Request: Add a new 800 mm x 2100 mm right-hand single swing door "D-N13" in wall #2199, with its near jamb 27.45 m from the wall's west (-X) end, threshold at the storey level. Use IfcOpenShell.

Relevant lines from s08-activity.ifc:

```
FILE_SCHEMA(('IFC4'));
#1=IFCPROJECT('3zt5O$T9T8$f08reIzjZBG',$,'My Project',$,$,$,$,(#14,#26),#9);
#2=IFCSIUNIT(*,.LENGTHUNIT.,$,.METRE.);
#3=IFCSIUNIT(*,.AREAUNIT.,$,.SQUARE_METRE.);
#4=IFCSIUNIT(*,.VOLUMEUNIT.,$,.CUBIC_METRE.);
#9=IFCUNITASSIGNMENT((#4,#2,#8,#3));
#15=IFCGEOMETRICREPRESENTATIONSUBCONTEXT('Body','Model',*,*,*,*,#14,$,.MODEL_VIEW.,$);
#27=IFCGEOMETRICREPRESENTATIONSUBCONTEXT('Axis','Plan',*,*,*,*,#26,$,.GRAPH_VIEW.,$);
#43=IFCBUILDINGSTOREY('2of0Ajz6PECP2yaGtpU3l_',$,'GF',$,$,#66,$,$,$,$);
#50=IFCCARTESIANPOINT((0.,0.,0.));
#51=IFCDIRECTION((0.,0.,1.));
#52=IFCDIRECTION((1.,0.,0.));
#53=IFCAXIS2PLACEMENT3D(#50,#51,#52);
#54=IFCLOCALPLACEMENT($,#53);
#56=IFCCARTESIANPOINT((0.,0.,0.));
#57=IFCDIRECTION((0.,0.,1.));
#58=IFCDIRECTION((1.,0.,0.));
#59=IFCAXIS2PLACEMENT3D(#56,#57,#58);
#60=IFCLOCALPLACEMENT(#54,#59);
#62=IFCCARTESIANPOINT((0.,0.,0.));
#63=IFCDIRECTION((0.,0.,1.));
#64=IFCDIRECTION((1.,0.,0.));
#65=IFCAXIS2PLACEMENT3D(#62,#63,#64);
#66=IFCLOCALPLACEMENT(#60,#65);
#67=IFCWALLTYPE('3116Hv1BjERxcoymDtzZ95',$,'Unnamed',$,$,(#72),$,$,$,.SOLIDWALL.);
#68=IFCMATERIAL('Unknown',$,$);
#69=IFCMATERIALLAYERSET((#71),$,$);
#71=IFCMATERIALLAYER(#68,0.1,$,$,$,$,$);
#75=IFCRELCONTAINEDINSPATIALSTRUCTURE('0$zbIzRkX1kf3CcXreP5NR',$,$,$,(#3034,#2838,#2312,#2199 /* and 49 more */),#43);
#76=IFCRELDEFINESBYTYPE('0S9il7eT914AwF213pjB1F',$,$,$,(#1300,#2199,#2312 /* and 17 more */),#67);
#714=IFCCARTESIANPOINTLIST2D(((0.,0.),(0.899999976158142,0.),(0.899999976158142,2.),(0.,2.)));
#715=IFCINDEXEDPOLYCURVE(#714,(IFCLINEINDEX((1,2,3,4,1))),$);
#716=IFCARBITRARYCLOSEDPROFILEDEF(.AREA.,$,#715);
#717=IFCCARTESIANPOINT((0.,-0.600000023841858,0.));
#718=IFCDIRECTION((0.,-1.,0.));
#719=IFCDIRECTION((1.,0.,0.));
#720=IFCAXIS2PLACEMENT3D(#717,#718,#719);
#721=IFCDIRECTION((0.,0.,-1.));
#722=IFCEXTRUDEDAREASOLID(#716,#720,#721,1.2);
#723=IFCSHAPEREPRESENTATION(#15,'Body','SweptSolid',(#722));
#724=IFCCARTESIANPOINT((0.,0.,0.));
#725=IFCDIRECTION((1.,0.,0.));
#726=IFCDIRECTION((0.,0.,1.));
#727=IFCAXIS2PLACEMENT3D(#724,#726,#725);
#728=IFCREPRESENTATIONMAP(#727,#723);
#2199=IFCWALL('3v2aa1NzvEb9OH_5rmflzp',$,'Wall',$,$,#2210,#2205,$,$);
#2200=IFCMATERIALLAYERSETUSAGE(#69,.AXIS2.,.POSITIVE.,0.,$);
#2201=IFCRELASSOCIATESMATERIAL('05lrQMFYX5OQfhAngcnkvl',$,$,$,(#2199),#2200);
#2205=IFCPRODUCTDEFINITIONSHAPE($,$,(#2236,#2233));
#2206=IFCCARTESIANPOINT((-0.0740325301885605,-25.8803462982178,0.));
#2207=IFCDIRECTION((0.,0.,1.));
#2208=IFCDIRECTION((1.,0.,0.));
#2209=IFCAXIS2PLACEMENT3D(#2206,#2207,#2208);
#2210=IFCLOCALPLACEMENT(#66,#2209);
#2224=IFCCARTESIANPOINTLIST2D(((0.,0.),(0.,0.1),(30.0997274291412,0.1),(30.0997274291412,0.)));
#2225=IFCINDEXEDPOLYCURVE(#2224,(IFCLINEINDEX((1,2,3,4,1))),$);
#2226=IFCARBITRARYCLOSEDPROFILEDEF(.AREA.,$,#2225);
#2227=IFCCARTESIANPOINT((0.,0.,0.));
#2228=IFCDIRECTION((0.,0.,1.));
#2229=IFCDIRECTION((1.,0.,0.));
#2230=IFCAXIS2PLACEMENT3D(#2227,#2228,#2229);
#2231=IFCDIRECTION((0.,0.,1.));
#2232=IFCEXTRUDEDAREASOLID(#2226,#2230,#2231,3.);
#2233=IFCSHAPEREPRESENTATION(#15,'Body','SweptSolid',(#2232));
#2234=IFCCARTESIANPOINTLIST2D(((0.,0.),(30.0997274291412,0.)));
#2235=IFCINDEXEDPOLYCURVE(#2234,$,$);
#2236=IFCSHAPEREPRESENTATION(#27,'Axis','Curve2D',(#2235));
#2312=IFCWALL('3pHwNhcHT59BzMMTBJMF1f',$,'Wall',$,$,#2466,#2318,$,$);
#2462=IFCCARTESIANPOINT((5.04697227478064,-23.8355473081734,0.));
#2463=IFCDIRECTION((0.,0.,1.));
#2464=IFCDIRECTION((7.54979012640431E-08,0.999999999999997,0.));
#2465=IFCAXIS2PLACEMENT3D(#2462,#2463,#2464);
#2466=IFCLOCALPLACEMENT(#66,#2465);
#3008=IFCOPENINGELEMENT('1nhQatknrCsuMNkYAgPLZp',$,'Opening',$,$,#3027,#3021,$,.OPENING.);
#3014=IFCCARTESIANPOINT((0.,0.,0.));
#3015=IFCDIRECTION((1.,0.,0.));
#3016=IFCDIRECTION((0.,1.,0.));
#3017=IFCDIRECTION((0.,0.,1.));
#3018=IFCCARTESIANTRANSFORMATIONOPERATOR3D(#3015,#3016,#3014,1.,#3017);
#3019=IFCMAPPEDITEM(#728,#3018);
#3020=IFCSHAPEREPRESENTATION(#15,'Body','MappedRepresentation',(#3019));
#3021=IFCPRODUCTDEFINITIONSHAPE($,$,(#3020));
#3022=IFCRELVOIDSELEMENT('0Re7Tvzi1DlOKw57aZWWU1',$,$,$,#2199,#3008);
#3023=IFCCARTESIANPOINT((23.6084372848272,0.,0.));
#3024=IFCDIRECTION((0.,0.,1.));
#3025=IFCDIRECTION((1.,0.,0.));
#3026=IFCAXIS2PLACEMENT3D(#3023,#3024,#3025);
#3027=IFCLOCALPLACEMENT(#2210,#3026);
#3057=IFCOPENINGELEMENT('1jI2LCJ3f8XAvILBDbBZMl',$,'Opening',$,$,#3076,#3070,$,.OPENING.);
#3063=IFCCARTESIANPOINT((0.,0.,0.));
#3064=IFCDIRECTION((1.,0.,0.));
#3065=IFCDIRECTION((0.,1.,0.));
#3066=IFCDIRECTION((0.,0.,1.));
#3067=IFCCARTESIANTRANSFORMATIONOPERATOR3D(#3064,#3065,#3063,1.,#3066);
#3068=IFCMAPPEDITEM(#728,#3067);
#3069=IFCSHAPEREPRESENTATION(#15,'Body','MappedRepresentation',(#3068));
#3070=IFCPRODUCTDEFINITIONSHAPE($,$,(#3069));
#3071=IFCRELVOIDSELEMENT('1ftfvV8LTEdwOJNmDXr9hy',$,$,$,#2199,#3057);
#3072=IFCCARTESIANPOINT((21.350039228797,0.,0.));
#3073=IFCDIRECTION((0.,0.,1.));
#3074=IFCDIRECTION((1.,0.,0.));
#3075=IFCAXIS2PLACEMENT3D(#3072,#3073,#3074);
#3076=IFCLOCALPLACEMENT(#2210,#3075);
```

```python
import numpy as np
import ifcopenshell
import ifcopenshell.api.feature
import ifcopenshell.api.geometry
import ifcopenshell.api.root
import ifcopenshell.api.spatial
import ifcopenshell.geom
import ifcopenshell.util.element
import ifcopenshell.util.placement
import ifcopenshell.util.representation
import ifcopenshell.util.shape
import ifcopenshell.util.unit

model = ifcopenshell.open("s08-activity.ifc")
unit_scale = ifcopenshell.util.unit.calculate_unit_scale(model)
settings = ifcopenshell.geom.settings()


def volume(element):
    """Net volume in cubic metres, openings subtracted."""
    shape = ifcopenshell.geom.create_shape(settings, element)
    return ifcopenshell.util.shape.get_volume(shape.geometry)


wall = model.by_guid("3v2aa1NzvEb9OH_5rmflzp")
storey = ifcopenshell.util.element.get_container(wall, ifc_class="IfcBuildingStorey")
context = ifcopenshell.util.representation.get_context(model, "Model", "Body", "MODEL_VIEW")
before = volume(wall)

width, height, from_end, sill = 0.8, 2.1, 27.45, 0.0  # metres

# The wall runs along its own X axis, and the end named is its -X end.
wall_shape = ifcopenshell.geom.create_shape(settings, wall)
x, y, z = ifcopenshell.util.shape.get_vertices(wall_shape.geometry).T
start = x.min() + from_end
face, thickness = float(y.min()), float(y.max() - y.min())
wall_matrix = ifcopenshell.util.placement.get_local_placement(wall.ObjectPlacement)
level = ifcopenshell.util.placement.get_local_placement(storey.ObjectPlacement)[2, 3]


def in_wall(x, y):
    """Placement at x, y metres in the wall's axes, at sill height."""
    matrix = wall_matrix.copy()
    matrix[:, 3] = wall_matrix @ np.array([x / unit_scale, y / unit_scale, 0.0, 1.0])
    matrix[2, 3] = level + sill / unit_scale
    return matrix


# Opening: a box that overshoots both wall faces by 50 mm.
opening = ifcopenshell.api.root.create_entity(model, ifc_class="IfcOpeningElement", predefined_type="OPENING")
box = ifcopenshell.api.geometry.add_wall_representation(
    model, context=context, length=width, height=height, thickness=thickness + 0.1
)
ifcopenshell.api.geometry.assign_representation(model, product=opening, representation=box)
ifcopenshell.api.geometry.edit_object_placement(model, product=opening, matrix=in_wall(start, face - 0.05), is_si=False)
ifcopenshell.api.feature.add_feature(model, feature=opening, element=wall)

door = ifcopenshell.api.root.create_entity(model, ifc_class="IfcDoor", name="D-N13", predefined_type="DOOR")
door.OverallWidth, door.OverallHeight = width / unit_scale, height / unit_scale
door.OperationType = "SINGLE_SWING_RIGHT"
body = ifcopenshell.api.geometry.add_door_representation(
    model,
    context=context,
    overall_width=door.OverallWidth,
    overall_height=door.OverallHeight,
    operation_type="SINGLE_SWING_RIGHT",
    lining_properties={"LiningDepth": thickness / unit_scale, "ThresholdDepth": thickness / unit_scale},
)
ifcopenshell.api.geometry.assign_representation(model, product=door, representation=body)
ifcopenshell.api.spatial.assign_container(model, products=[door], relating_structure=storey)
ifcopenshell.api.feature.add_filling(model, opening=opening, element=door)

# The lining spans the wall, so the door starts at the wall face.
ifcopenshell.api.geometry.edit_object_placement(model, product=door, matrix=in_wall(start, face), is_si=False)

after = volume(wall)

print(f"wall volume {before:.3f} -> {after:.3f} m3")

model.write("s08-activity-out.ifc")
```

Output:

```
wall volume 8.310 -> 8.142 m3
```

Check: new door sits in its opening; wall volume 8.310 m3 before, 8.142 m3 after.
